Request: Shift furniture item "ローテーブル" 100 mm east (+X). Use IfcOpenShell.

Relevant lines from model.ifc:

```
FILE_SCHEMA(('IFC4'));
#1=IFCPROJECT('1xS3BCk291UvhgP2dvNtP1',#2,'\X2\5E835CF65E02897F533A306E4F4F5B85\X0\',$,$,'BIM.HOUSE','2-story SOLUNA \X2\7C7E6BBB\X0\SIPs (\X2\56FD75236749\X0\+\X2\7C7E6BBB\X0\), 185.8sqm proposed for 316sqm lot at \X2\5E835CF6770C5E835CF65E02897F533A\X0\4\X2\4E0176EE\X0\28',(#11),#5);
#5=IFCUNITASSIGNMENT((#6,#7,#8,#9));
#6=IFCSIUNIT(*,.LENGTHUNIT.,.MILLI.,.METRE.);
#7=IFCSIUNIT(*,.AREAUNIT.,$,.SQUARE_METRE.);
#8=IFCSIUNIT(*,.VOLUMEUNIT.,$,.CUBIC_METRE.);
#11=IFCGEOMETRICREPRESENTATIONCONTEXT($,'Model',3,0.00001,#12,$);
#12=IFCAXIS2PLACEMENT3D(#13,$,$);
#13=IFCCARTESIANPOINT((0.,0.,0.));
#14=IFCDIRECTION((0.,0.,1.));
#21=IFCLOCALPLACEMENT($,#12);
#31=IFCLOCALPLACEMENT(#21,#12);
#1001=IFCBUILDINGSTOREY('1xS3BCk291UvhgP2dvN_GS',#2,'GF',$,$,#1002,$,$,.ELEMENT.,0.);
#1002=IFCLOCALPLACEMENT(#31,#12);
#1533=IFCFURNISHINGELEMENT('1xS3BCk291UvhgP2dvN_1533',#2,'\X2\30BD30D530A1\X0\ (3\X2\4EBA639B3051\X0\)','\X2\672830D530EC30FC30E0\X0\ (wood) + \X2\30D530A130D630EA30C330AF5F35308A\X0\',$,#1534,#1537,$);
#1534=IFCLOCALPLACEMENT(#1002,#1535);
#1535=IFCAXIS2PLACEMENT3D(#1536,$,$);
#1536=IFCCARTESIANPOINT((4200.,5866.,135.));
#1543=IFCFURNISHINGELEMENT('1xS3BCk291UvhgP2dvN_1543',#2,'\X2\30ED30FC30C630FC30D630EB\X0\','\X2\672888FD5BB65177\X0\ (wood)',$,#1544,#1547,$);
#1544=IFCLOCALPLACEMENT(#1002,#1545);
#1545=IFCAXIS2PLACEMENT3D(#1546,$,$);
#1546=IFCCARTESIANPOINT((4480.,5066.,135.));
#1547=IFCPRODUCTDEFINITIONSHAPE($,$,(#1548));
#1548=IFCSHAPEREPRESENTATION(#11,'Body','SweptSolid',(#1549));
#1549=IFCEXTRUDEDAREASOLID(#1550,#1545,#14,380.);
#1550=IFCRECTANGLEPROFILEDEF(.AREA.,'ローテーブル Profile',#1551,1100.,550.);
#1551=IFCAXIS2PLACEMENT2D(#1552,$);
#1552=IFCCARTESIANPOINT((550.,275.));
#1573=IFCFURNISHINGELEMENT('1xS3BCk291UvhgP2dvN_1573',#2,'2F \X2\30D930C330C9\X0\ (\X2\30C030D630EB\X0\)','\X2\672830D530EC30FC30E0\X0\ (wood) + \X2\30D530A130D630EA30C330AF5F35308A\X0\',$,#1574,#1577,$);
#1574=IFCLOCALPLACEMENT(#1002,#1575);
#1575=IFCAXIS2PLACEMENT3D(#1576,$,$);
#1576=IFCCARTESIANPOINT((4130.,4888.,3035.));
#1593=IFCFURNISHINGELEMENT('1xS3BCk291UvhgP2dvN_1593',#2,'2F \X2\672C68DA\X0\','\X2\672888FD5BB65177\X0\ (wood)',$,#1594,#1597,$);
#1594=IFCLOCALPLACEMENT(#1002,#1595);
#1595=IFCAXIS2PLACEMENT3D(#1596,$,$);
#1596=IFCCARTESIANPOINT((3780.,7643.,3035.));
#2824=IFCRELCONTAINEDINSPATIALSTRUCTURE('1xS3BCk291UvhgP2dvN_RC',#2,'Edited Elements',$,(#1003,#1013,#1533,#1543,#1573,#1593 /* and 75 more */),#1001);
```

```python
import ifcopenshell
import ifcopenshell.api.geometry
import ifcopenshell.util.placement
import ifcopenshell.util.unit

model = ifcopenshell.open("model.ifc")
unit_scale = ifcopenshell.util.unit.calculate_unit_scale(model)

item = model.by_id(1543)
matrix = ifcopenshell.util.placement.get_local_placement(item.ObjectPlacement)
matrix[0, 3] += 0.1 / unit_scale
ifcopenshell.api.geometry.edit_object_placement(model, product=item, matrix=matrix, is_si=False)

print(ifcopenshell.util.placement.get_local_placement(item.ObjectPlacement).round(3) + 0.0)

model.write("model_edited.ifc")
```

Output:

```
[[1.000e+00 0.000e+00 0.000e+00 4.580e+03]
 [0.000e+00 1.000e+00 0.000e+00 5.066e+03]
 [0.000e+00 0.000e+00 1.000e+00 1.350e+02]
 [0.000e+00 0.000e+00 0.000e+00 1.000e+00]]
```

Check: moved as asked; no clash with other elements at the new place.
